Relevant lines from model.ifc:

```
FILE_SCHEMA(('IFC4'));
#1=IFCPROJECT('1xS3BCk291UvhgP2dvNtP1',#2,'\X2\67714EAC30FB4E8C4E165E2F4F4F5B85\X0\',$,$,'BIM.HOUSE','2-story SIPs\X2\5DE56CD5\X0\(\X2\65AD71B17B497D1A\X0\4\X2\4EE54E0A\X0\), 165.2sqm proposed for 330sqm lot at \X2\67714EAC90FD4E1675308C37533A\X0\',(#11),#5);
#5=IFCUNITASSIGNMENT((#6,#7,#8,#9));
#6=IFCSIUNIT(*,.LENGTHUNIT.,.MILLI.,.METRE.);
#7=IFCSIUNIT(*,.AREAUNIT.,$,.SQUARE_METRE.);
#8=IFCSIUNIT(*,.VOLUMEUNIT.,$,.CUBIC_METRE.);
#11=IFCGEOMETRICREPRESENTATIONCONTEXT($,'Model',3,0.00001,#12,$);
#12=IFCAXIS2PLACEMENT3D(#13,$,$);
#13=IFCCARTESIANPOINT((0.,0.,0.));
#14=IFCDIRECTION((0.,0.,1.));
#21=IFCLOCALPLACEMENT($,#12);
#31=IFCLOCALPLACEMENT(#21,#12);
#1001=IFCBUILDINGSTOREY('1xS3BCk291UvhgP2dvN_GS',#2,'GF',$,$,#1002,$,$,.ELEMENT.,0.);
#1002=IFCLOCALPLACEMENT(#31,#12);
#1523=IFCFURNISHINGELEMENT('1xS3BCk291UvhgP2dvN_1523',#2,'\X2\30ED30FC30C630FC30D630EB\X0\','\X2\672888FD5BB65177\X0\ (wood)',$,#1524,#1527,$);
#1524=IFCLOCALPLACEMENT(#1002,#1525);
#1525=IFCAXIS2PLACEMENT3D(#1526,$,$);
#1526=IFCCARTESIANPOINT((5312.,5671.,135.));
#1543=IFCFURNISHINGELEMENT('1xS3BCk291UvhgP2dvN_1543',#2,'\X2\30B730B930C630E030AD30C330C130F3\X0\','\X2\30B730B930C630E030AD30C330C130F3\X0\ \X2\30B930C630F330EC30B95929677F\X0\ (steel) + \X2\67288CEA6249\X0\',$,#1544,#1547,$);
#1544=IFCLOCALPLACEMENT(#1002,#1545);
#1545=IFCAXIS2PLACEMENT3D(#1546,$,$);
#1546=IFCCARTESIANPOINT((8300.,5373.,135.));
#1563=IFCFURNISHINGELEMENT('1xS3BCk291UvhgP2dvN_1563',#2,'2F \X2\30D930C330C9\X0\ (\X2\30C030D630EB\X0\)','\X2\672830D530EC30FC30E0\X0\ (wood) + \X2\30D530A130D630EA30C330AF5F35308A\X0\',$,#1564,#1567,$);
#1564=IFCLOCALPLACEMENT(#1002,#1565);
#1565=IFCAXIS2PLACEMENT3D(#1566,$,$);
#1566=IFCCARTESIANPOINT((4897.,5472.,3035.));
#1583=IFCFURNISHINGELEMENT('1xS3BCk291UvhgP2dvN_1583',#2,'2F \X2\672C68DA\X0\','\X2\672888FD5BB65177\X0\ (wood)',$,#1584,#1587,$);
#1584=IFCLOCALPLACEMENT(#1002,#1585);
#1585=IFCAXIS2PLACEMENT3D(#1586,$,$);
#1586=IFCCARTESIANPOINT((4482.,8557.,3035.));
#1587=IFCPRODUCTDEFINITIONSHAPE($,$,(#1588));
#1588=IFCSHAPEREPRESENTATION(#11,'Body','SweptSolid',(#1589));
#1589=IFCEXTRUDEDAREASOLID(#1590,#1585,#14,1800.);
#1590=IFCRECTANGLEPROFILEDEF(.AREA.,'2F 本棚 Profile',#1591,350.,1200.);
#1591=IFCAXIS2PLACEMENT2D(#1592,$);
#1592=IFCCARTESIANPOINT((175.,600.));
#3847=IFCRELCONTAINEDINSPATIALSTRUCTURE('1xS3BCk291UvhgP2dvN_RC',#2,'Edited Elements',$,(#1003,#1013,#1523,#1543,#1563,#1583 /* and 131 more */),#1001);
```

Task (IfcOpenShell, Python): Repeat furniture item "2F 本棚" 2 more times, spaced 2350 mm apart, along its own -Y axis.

```python
import ifcopenshell
import ifcopenshell.api.geometry
import ifcopenshell.api.root
import ifcopenshell.util.element
import ifcopenshell.util.placement
import ifcopenshell.util.unit

model = ifcopenshell.open("model.ifc")
unit_scale = ifcopenshell.util.unit.calculate_unit_scale(model)


def reuse_history(source, copy):
    """copy_class also copies each property set's owner history, people and application; keep the originals."""
    for rel in copy.IsDefinedBy:
        if rel.is_a("IfcRelDefinesByProperties") and (history := rel.RelatingPropertyDefinition.OwnerHistory):
            rel.RelatingPropertyDefinition.OwnerHistory = source.OwnerHistory
            ifcopenshell.util.element.remove_deep2(model, history)


source = model.by_guid("1xS3BCk291UvhgP2dvN_1583")
base = ifcopenshell.util.placement.get_local_placement(source.ObjectPlacement)
step = -base[:3, 1] * 2.35 / unit_scale

for i in range(1, 3):
    copy = ifcopenshell.api.root.copy_class(model, product=source)
    copy.Representation = ifcopenshell.util.element.copy_deep(
        model, source.Representation, exclude=["IfcGeometricRepresentationContext", "IfcRepresentationMap"]
    )
    reuse_history(source, copy)
    matrix = base.copy()
    matrix[:3, 3] += i * step
    print("added at", matrix[:3, 3].round(3) + 0.0)
    ifcopenshell.api.geometry.edit_object_placement(model, product=copy, matrix=matrix, is_si=False)

model.write("model_edited.ifc")
```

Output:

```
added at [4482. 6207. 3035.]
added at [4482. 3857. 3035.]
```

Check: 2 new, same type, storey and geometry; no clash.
